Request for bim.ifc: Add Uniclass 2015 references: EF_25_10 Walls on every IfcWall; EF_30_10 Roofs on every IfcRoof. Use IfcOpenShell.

First a look at what the model holds.

```python
import ifcopenshell

model = ifcopenshell.open("bim.ifc")
print(model.schema)
print("classifications:", [c.Name for c in model.by_type("IfcClassification")])
for ifc_class in ("IfcDoor", "IfcRoof", "IfcStair", "IfcWall", "IfcWindow"):
    print(ifc_class, len(model.by_type(ifc_class)))
```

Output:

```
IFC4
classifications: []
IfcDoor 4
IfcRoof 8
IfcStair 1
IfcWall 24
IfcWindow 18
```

```python
import ifcopenshell
import ifcopenshell.api.classification

model = ifcopenshell.open("bim.ifc")

system = ifcopenshell.api.classification.add_classification(model, classification="Uniclass 2015")

codes = {
    "IfcWall": ("EF_25_10", "Walls"),
    "IfcRoof": ("EF_30_10", "Roofs"),
}
for ifc_class, (code, name) in codes.items():
    products = model.by_type(ifc_class)
    ifcopenshell.api.classification.add_reference(
        model, products=products, classification=system, identification=code, name=name
    )
    print(code, len(products))

model.write("bim_edited.ifc")
```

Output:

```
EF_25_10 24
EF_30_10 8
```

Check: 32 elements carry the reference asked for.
